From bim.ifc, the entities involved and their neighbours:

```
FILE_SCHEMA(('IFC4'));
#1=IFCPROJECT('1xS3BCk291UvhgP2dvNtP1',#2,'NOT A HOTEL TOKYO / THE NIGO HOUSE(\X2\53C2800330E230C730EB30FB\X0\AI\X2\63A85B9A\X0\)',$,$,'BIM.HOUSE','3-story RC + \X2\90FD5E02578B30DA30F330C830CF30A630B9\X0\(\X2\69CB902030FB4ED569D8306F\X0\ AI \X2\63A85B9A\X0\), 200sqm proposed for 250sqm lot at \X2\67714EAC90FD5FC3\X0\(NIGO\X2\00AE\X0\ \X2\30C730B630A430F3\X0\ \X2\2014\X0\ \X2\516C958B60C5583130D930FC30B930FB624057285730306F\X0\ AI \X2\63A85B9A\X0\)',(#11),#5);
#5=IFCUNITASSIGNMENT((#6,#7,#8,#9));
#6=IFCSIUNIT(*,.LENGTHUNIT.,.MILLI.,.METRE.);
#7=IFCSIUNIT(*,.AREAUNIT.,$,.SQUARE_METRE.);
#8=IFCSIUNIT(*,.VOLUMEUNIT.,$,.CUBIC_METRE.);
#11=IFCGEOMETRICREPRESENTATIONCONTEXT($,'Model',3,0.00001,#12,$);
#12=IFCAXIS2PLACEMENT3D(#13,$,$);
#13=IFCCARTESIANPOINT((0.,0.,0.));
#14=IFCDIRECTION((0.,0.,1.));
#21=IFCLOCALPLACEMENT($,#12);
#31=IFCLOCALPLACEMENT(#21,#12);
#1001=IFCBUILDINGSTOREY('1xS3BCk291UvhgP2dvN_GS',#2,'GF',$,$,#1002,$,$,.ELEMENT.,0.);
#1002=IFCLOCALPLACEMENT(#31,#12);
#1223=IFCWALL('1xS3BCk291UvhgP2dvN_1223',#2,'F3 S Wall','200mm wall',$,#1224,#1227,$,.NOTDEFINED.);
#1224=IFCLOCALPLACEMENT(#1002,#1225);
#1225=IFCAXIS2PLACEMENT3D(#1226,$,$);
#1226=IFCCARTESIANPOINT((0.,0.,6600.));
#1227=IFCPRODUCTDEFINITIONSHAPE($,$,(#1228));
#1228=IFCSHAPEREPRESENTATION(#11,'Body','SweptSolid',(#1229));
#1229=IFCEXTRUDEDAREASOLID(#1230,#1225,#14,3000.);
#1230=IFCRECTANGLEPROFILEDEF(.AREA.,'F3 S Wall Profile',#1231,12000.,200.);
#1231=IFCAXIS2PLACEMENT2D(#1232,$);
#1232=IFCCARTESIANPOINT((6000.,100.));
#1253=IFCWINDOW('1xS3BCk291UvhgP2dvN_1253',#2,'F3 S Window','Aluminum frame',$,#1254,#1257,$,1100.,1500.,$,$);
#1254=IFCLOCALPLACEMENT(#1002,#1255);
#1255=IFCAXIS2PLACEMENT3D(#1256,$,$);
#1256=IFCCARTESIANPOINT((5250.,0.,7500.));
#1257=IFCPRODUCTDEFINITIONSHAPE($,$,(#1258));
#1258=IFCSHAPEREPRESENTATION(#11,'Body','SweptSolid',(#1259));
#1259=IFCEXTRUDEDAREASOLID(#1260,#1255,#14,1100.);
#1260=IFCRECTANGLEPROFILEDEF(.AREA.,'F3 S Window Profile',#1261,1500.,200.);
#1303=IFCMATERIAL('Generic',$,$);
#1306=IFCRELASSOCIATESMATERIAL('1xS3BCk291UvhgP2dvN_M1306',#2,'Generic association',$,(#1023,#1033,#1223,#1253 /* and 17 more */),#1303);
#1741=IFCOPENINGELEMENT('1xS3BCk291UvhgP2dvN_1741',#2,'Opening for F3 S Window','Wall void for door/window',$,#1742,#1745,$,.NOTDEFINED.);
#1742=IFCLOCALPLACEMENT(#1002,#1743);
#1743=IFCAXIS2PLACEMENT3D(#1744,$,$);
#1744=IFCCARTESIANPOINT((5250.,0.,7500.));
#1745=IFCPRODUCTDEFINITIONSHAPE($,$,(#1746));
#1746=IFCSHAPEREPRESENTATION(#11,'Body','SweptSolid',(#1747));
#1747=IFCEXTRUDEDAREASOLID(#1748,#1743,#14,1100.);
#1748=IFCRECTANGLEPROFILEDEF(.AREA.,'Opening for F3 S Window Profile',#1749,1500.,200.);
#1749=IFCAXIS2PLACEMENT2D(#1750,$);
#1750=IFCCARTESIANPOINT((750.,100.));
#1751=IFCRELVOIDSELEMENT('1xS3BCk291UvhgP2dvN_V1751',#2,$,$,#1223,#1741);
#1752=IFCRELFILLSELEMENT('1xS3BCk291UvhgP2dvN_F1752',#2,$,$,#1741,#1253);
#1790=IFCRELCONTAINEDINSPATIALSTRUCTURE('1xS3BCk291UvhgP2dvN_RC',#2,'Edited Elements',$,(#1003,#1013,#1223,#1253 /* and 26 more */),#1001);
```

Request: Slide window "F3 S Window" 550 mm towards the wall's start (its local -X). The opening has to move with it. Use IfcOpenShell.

```python
import ifcopenshell
import ifcopenshell.api.geometry
import ifcopenshell.util.placement

model = ifcopenshell.open("bim.ifc")

window = model.by_guid("1xS3BCk291UvhgP2dvN_1253")
opening = window.FillsVoids[0].RelatingOpeningElement
wall = opening.VoidsElements[0].RelatingBuildingElement

wall_matrix = ifcopenshell.util.placement.get_local_placement(wall.ObjectPlacement)
shift = wall_matrix[:3, 0] * -550.0
before = ifcopenshell.util.placement.get_local_placement(window.ObjectPlacement)[:3, 3].copy()

# The window is not placed relative to its opening, so move both.
for product in (opening, window):
    matrix = ifcopenshell.util.placement.get_local_placement(product.ObjectPlacement)
    matrix[:3, 3] += shift
    ifcopenshell.api.geometry.edit_object_placement(model, product=product, matrix=matrix, is_si=False)

after = ifcopenshell.util.placement.get_local_placement(window.ObjectPlacement)[:3, 3]
print("window moved by", (after - before).round(3) + 0.0)

model.write("bim-out.ifc")
```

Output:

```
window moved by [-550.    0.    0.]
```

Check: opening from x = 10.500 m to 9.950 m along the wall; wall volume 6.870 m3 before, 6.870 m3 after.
